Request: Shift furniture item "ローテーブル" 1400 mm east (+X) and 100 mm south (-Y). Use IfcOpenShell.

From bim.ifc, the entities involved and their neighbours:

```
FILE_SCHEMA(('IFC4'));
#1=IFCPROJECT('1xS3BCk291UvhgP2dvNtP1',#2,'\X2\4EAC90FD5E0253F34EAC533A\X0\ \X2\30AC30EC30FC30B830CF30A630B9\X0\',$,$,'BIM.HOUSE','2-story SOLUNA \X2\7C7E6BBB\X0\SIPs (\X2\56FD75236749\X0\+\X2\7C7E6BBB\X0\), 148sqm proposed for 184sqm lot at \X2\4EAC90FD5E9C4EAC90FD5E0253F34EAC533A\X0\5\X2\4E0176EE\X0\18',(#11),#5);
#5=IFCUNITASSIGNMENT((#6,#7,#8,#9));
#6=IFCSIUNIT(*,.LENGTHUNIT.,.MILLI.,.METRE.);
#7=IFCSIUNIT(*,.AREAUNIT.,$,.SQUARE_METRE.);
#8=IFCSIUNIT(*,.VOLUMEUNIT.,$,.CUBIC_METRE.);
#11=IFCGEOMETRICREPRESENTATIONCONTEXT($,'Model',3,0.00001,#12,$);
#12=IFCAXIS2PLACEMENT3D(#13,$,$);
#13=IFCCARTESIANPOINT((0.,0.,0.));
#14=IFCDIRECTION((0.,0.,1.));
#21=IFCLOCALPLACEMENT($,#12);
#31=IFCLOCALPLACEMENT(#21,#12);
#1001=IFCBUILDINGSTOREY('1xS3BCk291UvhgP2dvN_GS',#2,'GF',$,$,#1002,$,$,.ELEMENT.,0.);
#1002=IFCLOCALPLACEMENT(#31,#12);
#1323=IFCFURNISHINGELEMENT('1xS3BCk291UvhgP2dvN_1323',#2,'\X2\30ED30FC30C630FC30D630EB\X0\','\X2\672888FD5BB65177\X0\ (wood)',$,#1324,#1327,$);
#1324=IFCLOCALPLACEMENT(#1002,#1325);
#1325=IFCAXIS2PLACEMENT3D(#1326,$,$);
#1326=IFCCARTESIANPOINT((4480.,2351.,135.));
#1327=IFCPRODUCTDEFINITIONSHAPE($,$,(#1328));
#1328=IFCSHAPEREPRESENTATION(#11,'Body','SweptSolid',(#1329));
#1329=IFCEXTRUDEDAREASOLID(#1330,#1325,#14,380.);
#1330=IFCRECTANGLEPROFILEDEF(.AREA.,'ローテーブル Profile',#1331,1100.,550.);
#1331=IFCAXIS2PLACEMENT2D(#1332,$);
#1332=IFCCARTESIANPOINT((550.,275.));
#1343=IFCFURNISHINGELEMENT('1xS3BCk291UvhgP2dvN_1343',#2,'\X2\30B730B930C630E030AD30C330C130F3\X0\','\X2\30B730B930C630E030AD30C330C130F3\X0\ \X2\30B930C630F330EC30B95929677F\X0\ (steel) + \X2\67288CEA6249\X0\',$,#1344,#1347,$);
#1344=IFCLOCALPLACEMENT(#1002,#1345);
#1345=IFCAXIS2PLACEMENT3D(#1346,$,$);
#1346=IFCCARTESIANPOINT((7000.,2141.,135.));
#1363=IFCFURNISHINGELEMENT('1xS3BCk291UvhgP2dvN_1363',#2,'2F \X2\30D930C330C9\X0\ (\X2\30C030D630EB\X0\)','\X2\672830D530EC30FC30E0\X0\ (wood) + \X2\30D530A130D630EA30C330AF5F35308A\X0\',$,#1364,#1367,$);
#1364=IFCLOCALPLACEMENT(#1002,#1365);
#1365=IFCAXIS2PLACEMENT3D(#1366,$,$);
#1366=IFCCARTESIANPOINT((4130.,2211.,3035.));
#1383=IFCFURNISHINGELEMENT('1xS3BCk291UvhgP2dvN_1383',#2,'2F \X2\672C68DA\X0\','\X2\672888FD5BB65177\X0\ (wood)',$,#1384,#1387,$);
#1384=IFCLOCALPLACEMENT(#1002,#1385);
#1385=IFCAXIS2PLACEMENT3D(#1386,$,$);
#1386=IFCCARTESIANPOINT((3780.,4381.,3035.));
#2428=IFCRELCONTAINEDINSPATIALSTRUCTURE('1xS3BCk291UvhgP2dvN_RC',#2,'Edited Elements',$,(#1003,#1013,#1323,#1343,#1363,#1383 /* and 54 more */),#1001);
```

```python
import ifcopenshell
import ifcopenshell.api.geometry
import ifcopenshell.util.placement

model = ifcopenshell.open("bim.ifc")

item = model.by_guid("1xS3BCk291UvhgP2dvN_1323")
matrix = ifcopenshell.util.placement.get_local_placement(item.ObjectPlacement)
matrix[0, 3] += 1400.0
matrix[1, 3] -= 100.0
ifcopenshell.api.geometry.edit_object_placement(model, product=item, matrix=matrix, is_si=False)

print(ifcopenshell.util.placement.get_local_placement(item.ObjectPlacement).round(3) + 0.0)

model.write("bim_v2.ifc")
```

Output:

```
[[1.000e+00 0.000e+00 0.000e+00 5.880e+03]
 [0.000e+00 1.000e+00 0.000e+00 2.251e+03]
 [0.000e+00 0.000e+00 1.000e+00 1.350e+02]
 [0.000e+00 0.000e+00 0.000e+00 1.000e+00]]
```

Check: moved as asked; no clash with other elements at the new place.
